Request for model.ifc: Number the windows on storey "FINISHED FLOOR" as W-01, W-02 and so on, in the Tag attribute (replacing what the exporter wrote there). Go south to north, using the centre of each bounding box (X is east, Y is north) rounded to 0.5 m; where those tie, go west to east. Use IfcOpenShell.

First a look at what the model holds.

```python
import ifcopenshell
import ifcopenshell.util.element
import ifcopenshell.util.placement

model = ifcopenshell.open("model.ifc")
print(model.schema)
storey = next(s for s in model.by_type("IfcBuildingStorey") if s.Name == "FINISHED FLOOR")
windows = [e for e in ifcopenshell.util.element.get_decomposition(storey) if e.is_a("IfcWindow")]
for e in sorted(windows, key=lambda e: e.id()):
    origin = ifcopenshell.util.placement.get_local_placement(e.ObjectPlacement)[:3, 3]
    print(e.id(), e.Tag, e.Name, origin.round(2) + 0.0, sep=" | ")
```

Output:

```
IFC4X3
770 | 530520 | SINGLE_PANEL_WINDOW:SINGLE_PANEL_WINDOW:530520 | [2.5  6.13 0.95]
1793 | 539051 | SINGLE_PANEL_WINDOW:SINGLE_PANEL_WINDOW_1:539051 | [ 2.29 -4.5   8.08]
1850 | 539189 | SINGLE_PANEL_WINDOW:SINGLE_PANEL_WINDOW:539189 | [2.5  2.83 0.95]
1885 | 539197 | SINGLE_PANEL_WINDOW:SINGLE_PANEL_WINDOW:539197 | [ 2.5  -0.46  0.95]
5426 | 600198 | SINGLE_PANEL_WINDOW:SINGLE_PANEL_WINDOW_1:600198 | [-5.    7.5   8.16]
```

```python
import ifcopenshell
import ifcopenshell.geom
import ifcopenshell.util.element
import ifcopenshell.util.shape

model = ifcopenshell.open("model.ifc")
settings = ifcopenshell.geom.settings()
settings.set("use-world-coords", True)


def centre(element):
    shape = ifcopenshell.geom.create_shape(settings, element)
    return ifcopenshell.util.shape.get_bbox_centroid(shape.geometry)


storey = next(s for s in model.by_type("IfcBuildingStorey") if s.Name == "FINISHED FLOOR")
windows = [e for e in ifcopenshell.util.element.get_decomposition(storey) if e.is_a("IfcWindow")]

# Insertion points can sit at a corner or the storey origin, so sort by the geometry (in metres).
centres = {e: centre(e) for e in windows}
windows.sort(key=lambda e: (round(centres[e][1] / 0.5), centres[e][0]))

for i, e in enumerate(windows, start=1):
    number = f"W-{i:02d}"
    e.Tag = number
    print(e.id(), number)

model.write("model-out.ifc")
```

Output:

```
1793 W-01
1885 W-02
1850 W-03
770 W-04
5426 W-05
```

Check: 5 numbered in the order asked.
